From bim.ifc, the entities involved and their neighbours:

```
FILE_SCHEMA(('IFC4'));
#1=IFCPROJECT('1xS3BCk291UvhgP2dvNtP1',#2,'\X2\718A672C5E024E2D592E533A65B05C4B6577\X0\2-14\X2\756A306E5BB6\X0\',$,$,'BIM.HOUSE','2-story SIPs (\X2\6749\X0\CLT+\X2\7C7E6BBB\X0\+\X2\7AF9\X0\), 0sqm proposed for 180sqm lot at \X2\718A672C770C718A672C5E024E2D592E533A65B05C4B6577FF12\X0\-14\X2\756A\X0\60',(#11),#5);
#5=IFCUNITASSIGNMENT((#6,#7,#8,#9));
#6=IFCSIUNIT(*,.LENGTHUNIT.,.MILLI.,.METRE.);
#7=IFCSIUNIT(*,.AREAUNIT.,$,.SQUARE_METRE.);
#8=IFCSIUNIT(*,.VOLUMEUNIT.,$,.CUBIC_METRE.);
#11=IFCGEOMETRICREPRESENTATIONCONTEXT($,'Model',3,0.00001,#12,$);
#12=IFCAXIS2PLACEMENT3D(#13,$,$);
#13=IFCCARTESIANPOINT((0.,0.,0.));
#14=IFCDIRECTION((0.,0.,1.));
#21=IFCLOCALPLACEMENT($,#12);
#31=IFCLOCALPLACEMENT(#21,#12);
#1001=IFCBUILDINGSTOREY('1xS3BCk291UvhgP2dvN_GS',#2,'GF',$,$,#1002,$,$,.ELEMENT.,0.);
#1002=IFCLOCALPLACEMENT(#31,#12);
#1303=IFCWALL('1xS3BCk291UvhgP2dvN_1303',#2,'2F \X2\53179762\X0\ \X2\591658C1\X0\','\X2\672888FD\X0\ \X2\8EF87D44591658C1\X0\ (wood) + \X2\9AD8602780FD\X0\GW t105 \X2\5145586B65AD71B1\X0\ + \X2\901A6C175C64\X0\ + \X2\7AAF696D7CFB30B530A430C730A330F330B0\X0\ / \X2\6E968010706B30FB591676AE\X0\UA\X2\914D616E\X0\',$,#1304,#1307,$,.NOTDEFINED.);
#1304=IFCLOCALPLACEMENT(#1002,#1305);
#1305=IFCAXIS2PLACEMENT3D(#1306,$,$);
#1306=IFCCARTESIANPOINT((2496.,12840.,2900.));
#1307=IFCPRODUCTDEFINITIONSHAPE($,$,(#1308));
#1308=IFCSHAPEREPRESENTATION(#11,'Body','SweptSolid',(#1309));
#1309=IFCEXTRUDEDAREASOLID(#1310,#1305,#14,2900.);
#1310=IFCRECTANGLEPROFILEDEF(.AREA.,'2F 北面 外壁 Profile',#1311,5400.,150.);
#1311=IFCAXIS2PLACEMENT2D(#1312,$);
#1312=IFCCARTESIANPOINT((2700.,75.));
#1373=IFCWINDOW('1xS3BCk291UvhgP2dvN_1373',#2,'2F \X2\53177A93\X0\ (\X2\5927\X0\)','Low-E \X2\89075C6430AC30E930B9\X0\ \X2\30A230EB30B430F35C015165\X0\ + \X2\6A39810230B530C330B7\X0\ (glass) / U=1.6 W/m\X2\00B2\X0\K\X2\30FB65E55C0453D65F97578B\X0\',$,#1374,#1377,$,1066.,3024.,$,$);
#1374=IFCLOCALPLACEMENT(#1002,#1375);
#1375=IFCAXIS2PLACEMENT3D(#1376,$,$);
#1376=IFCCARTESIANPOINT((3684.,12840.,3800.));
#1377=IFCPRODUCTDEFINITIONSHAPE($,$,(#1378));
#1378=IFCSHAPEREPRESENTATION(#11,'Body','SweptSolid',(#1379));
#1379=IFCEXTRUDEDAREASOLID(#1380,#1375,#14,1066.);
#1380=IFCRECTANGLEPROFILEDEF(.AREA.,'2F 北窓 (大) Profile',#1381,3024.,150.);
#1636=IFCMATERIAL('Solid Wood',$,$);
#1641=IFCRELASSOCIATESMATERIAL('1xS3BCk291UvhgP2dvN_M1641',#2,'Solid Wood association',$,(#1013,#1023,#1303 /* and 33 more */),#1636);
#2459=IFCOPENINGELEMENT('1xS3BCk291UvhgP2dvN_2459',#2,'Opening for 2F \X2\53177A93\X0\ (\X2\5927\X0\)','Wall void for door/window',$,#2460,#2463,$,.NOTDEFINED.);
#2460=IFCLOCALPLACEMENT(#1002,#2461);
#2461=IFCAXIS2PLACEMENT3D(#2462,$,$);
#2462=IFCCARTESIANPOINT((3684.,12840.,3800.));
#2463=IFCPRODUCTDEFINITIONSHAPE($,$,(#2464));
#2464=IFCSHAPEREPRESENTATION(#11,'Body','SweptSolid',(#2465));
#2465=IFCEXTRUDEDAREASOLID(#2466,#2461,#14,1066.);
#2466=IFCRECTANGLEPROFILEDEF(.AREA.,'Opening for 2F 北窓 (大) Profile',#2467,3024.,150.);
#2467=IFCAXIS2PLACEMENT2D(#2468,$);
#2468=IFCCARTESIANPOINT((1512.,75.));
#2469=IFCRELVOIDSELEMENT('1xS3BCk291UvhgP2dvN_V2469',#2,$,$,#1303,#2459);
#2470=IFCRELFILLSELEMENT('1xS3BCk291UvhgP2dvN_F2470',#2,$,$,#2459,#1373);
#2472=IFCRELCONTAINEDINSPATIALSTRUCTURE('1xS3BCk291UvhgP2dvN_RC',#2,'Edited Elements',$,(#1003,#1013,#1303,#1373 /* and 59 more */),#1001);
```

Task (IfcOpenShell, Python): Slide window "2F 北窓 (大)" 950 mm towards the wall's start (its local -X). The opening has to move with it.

```python
import ifcopenshell
import ifcopenshell.api.geometry
import ifcopenshell.util.placement
import ifcopenshell.util.unit

model = ifcopenshell.open("bim.ifc")
unit_scale = ifcopenshell.util.unit.calculate_unit_scale(model)

window = model.by_guid("1xS3BCk291UvhgP2dvN_1373")
opening = window.FillsVoids[0].RelatingOpeningElement
wall = opening.VoidsElements[0].RelatingBuildingElement

wall_matrix = ifcopenshell.util.placement.get_local_placement(wall.ObjectPlacement)
shift = wall_matrix[:3, 0] * -0.95 / unit_scale
before = ifcopenshell.util.placement.get_local_placement(window.ObjectPlacement)[:3, 3].copy()

# The window is not placed relative to its opening, so move both.
for product in (opening, window):
    matrix = ifcopenshell.util.placement.get_local_placement(product.ObjectPlacement)
    matrix[:3, 3] += shift
    ifcopenshell.api.geometry.edit_object_placement(model, product=product, matrix=matrix, is_si=False)

after = ifcopenshell.util.placement.get_local_placement(window.ObjectPlacement)[:3, 3]
print("window moved by", (after - before).round(3) + 0.0)

model.write("bim_v2.ifc")
```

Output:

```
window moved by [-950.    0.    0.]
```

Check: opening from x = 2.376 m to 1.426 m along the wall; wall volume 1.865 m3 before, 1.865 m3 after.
